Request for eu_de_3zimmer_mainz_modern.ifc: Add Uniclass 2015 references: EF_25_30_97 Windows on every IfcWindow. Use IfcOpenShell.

First a look at what the model holds.

```python
import ifcopenshell

model = ifcopenshell.open("eu_de_3zimmer_mainz_modern.ifc")
print(model.schema)
print("classifications:", [c.Name for c in model.by_type("IfcClassification")])
for ifc_class in ("IfcDoor", "IfcRoof", "IfcStair", "IfcWall", "IfcWindow"):
    print(ifc_class, len(model.by_type(ifc_class)))
```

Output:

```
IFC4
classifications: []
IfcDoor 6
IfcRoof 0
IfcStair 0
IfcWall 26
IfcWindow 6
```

```python
import ifcopenshell
import ifcopenshell.api.classification

model = ifcopenshell.open("eu_de_3zimmer_mainz_modern.ifc")

system = ifcopenshell.api.classification.add_classification(model, classification="Uniclass 2015")

codes = {
    "IfcWindow": ("EF_25_30_97", "Windows"),
}
for ifc_class, (code, name) in codes.items():
    products = model.by_type(ifc_class)
    ifcopenshell.api.classification.add_reference(
        model, products=products, classification=system, identification=code, name=name
    )
    print(code, len(products))

model.write("eu_de_3zimmer_mainz_modern_updated.ifc")
```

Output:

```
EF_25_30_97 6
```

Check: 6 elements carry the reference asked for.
